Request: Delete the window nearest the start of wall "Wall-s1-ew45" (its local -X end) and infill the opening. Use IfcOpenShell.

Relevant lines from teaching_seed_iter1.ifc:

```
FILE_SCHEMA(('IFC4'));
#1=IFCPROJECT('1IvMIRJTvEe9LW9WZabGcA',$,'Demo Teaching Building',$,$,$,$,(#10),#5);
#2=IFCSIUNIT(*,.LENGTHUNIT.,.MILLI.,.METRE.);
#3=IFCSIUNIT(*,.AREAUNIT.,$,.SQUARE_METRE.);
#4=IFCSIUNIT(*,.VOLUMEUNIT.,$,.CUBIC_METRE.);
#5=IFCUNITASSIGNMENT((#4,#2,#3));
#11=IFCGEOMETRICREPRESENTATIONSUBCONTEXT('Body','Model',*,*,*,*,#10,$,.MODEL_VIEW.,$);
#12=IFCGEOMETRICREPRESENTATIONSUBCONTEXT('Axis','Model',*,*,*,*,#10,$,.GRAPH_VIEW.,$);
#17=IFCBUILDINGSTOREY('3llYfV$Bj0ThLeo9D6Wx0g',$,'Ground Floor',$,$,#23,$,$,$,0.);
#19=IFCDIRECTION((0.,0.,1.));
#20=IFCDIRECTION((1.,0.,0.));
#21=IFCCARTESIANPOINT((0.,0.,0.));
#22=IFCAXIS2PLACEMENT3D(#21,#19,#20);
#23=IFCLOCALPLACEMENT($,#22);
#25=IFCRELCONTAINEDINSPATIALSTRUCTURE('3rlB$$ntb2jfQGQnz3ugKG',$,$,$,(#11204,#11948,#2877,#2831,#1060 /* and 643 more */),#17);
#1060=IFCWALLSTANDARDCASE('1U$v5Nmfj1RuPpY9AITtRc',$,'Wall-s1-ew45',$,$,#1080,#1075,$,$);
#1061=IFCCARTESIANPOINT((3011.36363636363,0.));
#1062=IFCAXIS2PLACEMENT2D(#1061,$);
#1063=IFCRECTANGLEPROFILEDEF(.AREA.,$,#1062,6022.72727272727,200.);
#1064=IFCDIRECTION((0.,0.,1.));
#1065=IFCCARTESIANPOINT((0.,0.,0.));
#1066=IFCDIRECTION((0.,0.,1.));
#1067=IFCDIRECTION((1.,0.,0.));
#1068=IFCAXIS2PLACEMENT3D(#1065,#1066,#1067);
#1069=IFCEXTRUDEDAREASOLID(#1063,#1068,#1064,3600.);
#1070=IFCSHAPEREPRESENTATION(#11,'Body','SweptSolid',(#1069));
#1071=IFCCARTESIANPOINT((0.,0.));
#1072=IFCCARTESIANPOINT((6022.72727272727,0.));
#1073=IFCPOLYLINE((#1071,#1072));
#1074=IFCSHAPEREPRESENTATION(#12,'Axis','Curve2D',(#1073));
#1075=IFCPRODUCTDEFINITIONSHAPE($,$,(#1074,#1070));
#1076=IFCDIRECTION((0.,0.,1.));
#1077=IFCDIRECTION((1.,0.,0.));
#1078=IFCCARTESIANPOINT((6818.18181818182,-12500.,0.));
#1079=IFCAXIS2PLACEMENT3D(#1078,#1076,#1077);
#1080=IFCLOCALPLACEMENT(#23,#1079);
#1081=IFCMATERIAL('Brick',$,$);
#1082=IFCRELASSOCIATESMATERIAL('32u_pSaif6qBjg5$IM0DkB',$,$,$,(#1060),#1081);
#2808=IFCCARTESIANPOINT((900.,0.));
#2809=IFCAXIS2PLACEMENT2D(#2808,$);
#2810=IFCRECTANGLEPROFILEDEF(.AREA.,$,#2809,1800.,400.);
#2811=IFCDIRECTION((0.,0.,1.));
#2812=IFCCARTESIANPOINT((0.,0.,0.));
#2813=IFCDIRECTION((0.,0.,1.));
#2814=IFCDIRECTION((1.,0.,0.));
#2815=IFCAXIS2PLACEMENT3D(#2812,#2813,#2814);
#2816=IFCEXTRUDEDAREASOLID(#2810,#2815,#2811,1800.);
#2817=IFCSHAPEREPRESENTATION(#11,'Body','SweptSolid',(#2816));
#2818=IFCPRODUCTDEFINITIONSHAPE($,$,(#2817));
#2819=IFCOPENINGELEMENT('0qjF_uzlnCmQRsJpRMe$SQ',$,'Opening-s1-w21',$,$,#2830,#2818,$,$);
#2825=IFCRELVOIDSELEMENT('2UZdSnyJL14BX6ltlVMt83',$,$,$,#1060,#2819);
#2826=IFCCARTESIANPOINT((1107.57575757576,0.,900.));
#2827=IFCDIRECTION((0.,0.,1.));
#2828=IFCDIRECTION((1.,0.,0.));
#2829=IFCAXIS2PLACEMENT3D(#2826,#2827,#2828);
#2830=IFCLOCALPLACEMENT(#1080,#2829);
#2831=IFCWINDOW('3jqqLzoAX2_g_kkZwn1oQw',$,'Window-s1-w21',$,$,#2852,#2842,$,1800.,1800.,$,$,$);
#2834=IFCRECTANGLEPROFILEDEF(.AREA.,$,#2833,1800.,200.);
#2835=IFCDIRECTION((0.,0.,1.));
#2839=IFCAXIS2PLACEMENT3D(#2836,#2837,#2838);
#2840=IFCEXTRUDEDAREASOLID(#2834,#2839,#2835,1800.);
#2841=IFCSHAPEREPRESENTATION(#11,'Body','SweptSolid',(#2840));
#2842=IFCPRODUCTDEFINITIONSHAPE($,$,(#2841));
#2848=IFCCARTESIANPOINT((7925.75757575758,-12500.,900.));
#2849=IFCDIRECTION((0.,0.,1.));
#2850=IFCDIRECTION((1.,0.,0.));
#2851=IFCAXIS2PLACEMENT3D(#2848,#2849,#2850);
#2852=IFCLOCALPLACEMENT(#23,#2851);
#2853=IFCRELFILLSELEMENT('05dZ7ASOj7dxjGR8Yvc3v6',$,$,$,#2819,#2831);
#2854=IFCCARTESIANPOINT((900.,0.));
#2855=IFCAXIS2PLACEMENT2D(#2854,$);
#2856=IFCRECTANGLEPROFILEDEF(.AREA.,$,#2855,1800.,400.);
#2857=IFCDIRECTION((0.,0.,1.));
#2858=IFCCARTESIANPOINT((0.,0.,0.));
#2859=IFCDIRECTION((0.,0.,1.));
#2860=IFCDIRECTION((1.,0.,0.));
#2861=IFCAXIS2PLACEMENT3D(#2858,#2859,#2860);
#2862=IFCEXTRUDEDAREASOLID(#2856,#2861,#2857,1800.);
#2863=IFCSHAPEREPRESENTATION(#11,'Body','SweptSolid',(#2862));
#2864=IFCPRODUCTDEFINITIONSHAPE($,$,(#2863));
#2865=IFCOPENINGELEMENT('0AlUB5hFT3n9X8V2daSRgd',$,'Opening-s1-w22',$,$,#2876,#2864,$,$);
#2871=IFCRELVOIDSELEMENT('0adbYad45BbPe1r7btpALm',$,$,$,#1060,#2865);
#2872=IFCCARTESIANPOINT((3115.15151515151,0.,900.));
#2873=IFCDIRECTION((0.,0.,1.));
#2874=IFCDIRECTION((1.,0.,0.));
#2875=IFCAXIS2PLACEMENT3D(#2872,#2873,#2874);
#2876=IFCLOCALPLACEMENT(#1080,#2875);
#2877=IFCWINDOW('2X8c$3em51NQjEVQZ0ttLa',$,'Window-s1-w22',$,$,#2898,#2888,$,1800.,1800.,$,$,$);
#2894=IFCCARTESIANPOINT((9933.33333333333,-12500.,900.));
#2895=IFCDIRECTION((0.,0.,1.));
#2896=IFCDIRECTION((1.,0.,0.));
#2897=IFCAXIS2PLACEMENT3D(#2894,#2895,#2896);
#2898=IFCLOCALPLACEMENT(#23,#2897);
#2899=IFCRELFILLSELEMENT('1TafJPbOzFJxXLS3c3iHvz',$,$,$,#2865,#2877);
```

```python
import ifcopenshell
import ifcopenshell.api.feature
import ifcopenshell.api.root
import ifcopenshell.geom
import ifcopenshell.util.shape

model = ifcopenshell.open("teaching_seed_iter1.ifc")
settings = ifcopenshell.geom.settings()


def volume(element):
    """Net volume in cubic metres, openings subtracted."""
    shape = ifcopenshell.geom.create_shape(settings, element)
    return ifcopenshell.util.shape.get_volume(shape.geometry)


window = model.by_id(2831)
opening = window.FillsVoids[0].RelatingOpeningElement
wall = opening.VoidsElements[0].RelatingBuildingElement
before = volume(wall)

ifcopenshell.api.root.remove_product(model, product=window)
ifcopenshell.api.feature.remove_feature(model, feature=opening)

after = volume(wall)

print(f"wall volume {before:.3f} -> {after:.3f} m3")

model.write("teaching_seed_iter1-out.ifc")
```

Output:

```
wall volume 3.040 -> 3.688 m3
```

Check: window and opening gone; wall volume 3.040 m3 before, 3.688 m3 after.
